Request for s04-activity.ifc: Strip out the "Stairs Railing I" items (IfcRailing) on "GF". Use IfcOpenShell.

First a look at what the model holds.

```python
import ifcopenshell
import ifcopenshell.util.element

model = ifcopenshell.open("s04-activity.ifc")
print(model.schema)
storey = next(s for s in model.by_type("IfcBuildingStorey") if s.Name == "GF")
railings = [e for e in ifcopenshell.util.element.get_decomposition(storey) if e.is_a("IfcRailing")]
seen = {}
for e in railings:
    element_type = ifcopenshell.util.element.get_type(e)
    name = element_type.Name if element_type not in (None, e) else None
    seen[name] = seen.get(name, 0) + 1
for name, count in sorted(seen.items(), key=str):
    print(count, "x", name)
```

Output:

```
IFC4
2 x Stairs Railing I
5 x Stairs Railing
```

```python
import ifcopenshell
import ifcopenshell.api.root
import ifcopenshell.util.element

model = ifcopenshell.open("s04-activity.ifc")

storey = next(s for s in model.by_type("IfcBuildingStorey") if s.Name == "GF")
railings = [e for e in ifcopenshell.util.element.get_decomposition(storey) if e.is_a("IfcRailing")]
targets = [e for e in railings if (t := ifcopenshell.util.element.get_type(e)) not in (None, e) and t.Name == "Stairs Railing I"]

for e in targets:
    ifcopenshell.api.root.remove_product(model, product=e)
print(len(targets), "removed")

model.write("s04-activity_updated.ifc")
```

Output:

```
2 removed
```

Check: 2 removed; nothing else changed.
